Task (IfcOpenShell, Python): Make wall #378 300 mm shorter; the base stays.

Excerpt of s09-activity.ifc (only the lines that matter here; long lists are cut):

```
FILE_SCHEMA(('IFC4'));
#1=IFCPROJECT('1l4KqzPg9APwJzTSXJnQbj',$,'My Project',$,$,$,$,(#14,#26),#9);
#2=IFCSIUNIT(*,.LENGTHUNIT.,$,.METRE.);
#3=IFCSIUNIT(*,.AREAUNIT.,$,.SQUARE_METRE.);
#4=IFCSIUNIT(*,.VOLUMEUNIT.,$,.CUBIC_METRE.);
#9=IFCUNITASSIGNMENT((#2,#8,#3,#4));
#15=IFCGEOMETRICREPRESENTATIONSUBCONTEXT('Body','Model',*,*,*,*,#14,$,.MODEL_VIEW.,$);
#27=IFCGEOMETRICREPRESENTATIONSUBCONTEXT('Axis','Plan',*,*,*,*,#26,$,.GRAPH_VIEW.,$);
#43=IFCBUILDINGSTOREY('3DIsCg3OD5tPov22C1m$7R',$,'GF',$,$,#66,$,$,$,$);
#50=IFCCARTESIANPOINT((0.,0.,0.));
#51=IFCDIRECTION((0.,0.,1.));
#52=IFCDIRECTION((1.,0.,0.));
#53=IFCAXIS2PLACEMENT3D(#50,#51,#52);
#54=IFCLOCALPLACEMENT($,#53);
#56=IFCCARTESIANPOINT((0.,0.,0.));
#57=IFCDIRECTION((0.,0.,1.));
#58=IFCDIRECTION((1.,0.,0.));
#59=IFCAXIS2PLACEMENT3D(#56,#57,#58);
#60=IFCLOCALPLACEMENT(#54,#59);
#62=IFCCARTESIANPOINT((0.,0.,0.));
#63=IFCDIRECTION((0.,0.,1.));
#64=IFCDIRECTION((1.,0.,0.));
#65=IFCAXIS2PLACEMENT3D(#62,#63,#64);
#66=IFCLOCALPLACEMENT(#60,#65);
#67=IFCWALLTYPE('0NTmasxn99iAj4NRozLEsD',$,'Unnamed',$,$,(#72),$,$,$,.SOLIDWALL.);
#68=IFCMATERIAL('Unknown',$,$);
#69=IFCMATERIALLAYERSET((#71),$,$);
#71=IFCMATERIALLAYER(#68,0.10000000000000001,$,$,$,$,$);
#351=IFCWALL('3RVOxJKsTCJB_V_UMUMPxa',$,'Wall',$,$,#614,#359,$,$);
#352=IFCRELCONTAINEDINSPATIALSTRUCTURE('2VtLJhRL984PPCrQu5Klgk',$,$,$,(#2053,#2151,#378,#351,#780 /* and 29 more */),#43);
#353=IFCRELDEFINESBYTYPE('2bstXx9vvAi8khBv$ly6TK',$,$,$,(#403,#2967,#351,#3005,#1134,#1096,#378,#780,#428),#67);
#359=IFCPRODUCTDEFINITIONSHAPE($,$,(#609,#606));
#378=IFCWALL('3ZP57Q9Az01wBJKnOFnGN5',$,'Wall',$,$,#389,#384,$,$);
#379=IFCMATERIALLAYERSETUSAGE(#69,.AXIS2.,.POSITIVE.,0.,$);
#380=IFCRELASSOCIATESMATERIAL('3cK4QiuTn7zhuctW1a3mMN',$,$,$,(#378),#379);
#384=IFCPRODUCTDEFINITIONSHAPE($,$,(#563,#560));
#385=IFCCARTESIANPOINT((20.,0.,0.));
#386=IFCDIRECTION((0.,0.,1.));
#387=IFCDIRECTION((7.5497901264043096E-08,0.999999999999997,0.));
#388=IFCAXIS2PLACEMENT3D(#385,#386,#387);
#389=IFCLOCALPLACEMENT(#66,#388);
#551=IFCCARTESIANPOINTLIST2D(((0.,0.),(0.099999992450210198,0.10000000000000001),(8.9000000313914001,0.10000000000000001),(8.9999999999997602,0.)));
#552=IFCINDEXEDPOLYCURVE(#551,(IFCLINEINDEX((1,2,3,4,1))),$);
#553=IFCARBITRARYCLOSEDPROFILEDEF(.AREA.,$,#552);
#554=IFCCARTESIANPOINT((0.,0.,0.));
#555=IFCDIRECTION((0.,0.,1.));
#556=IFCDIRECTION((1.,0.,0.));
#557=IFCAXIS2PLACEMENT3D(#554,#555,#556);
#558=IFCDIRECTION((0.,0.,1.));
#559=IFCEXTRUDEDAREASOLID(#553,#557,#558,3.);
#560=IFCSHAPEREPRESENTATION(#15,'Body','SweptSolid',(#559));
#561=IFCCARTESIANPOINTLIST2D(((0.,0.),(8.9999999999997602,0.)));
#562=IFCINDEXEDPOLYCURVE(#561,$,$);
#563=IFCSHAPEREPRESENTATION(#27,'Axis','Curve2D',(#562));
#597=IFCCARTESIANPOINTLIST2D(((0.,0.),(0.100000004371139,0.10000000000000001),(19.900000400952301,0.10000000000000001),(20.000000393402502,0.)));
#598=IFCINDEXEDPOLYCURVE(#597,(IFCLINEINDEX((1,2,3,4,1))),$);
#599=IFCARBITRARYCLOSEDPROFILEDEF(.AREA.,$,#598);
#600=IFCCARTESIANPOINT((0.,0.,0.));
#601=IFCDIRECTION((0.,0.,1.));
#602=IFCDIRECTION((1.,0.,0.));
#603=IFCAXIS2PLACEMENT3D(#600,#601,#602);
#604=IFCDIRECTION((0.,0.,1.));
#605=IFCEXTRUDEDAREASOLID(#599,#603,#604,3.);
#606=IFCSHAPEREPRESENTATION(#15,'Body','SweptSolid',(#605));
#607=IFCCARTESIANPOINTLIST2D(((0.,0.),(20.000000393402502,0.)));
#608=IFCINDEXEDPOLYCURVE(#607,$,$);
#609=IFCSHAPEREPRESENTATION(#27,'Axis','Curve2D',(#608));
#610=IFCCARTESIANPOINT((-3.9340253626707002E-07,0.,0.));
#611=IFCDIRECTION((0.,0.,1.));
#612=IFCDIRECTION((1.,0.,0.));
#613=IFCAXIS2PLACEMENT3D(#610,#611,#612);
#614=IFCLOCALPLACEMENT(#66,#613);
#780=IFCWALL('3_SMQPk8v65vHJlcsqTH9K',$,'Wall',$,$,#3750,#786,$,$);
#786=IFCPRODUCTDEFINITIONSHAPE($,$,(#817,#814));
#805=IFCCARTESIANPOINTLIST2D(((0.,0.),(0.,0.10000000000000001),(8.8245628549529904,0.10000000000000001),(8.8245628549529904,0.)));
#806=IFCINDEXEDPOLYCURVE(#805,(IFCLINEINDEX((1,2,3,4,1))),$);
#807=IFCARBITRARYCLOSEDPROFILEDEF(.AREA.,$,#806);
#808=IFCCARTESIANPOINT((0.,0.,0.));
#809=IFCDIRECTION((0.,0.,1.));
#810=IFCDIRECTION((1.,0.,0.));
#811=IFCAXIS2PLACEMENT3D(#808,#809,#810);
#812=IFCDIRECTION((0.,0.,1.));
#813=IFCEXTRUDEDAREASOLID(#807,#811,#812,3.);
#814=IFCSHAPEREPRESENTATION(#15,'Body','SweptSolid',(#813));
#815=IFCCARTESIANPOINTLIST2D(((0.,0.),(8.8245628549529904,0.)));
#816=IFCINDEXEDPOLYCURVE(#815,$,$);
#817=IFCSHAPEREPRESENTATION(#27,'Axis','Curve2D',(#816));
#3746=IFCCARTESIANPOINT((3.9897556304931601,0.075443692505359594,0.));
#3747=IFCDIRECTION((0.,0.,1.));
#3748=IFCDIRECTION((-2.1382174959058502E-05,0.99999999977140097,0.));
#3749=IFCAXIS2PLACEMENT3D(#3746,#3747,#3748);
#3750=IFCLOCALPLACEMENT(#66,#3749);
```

```python
import ifcopenshell
import ifcopenshell.geom
import ifcopenshell.util.representation
import ifcopenshell.util.shape

model = ifcopenshell.open("s09-activity.ifc")
settings = ifcopenshell.geom.settings()


def volume(element):
    """Net volume in cubic metres, openings subtracted."""
    shape = ifcopenshell.geom.create_shape(settings, element)
    return ifcopenshell.util.shape.get_volume(shape.geometry)


wall = model.by_guid("3ZP57Q9Az01wBJKnOFnGN5")
before = volume(wall)

body = ifcopenshell.util.representation.get_representation(wall, "Model", "Body")
solid = body.Items[0]
old_height = solid.Depth
solid.Depth -= 0.3
after = volume(wall)

print(f"height {old_height:g} -> {solid.Depth:g}, volume {before:.3f} -> {after:.3f} m3")

model.write("s09-activity-out.ifc")
```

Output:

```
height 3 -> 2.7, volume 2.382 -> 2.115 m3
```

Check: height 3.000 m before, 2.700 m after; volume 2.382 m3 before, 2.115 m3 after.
